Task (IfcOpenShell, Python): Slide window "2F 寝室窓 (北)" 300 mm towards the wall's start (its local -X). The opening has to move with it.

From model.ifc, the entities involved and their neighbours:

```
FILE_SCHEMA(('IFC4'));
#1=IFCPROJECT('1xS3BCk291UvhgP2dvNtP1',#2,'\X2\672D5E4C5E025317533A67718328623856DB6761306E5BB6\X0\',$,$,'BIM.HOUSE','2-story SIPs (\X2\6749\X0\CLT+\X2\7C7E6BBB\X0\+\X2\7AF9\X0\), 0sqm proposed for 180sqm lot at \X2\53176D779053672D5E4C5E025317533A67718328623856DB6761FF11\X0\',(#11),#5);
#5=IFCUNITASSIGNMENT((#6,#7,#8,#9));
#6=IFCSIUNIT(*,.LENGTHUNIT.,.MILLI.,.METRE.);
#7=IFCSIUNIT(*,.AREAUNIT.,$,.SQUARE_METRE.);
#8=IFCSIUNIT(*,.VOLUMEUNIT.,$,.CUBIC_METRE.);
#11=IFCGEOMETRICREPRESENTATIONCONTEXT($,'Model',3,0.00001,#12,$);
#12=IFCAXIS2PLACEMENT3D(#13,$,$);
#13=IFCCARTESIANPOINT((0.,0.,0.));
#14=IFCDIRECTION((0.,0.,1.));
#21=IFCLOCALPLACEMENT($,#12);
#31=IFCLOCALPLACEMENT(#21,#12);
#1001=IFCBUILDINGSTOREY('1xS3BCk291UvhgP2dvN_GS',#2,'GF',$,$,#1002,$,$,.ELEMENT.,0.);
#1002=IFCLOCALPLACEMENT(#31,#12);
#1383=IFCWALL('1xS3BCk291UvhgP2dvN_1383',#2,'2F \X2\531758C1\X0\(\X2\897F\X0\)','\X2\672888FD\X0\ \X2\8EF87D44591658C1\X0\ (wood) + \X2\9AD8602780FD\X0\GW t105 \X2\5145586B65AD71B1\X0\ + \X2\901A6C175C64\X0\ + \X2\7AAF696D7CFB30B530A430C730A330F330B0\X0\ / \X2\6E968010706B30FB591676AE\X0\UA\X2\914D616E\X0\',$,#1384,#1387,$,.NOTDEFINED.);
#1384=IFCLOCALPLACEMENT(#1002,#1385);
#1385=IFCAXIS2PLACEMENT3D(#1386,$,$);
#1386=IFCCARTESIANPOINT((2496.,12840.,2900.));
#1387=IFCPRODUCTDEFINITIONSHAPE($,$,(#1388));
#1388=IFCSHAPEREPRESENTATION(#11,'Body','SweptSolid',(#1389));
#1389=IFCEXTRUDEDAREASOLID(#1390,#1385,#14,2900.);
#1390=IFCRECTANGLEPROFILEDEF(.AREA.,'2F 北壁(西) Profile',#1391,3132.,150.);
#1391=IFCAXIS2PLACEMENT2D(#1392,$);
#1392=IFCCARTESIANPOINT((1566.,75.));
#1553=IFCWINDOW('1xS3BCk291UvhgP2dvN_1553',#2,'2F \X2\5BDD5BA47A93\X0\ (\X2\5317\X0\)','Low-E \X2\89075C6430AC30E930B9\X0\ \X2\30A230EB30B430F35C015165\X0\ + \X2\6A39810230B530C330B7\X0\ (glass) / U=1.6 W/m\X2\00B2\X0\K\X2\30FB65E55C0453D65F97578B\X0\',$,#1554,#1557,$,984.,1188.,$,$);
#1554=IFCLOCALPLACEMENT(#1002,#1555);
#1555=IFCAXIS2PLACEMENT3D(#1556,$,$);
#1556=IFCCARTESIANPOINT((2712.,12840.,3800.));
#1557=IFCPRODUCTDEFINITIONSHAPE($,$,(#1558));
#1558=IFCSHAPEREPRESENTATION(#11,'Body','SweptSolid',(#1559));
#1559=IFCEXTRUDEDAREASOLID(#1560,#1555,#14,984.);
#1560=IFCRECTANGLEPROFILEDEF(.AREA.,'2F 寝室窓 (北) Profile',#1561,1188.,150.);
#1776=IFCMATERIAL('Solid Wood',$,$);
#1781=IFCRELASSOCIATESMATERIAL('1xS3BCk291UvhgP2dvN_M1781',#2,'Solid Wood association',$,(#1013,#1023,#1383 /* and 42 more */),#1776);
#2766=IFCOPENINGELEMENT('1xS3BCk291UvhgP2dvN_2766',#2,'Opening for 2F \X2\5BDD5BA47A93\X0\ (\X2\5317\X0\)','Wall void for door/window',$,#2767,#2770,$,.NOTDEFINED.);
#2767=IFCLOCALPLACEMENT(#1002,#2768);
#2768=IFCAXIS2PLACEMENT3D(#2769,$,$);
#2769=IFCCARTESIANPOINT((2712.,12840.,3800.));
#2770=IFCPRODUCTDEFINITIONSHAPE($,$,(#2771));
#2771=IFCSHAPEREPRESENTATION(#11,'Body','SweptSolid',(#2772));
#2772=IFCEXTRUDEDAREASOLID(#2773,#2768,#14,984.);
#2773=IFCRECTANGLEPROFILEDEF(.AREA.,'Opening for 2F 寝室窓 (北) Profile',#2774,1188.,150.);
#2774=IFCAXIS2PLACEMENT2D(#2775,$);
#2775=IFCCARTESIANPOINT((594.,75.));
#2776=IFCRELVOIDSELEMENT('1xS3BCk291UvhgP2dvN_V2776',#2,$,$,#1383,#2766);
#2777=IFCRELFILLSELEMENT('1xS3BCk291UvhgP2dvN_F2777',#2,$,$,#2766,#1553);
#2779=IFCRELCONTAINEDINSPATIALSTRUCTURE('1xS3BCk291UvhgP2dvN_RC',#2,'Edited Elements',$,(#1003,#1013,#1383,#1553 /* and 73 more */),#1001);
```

```python
import ifcopenshell
import ifcopenshell.api.geometry
import ifcopenshell.util.placement

model = ifcopenshell.open("model.ifc")

window = model.by_guid("1xS3BCk291UvhgP2dvN_1553")
opening = window.FillsVoids[0].RelatingOpeningElement
wall = opening.VoidsElements[0].RelatingBuildingElement

wall_matrix = ifcopenshell.util.placement.get_local_placement(wall.ObjectPlacement)
shift = wall_matrix[:3, 0] * -300.0
before = ifcopenshell.util.placement.get_local_placement(window.ObjectPlacement)[:3, 3].copy()

# The window is not placed relative to its opening, so move both.
for product in (opening, window):
    matrix = ifcopenshell.util.placement.get_local_placement(product.ObjectPlacement)
    matrix[:3, 3] += shift
    ifcopenshell.api.geometry.edit_object_placement(model, product=product, matrix=matrix, is_si=False)

after = ifcopenshell.util.placement.get_local_placement(window.ObjectPlacement)[:3, 3]
print("window moved by", (after - before).round(3) + 0.0)

model.write("model_updated.ifc")
```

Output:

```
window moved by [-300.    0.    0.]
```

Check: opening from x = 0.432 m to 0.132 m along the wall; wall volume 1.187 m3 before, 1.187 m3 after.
